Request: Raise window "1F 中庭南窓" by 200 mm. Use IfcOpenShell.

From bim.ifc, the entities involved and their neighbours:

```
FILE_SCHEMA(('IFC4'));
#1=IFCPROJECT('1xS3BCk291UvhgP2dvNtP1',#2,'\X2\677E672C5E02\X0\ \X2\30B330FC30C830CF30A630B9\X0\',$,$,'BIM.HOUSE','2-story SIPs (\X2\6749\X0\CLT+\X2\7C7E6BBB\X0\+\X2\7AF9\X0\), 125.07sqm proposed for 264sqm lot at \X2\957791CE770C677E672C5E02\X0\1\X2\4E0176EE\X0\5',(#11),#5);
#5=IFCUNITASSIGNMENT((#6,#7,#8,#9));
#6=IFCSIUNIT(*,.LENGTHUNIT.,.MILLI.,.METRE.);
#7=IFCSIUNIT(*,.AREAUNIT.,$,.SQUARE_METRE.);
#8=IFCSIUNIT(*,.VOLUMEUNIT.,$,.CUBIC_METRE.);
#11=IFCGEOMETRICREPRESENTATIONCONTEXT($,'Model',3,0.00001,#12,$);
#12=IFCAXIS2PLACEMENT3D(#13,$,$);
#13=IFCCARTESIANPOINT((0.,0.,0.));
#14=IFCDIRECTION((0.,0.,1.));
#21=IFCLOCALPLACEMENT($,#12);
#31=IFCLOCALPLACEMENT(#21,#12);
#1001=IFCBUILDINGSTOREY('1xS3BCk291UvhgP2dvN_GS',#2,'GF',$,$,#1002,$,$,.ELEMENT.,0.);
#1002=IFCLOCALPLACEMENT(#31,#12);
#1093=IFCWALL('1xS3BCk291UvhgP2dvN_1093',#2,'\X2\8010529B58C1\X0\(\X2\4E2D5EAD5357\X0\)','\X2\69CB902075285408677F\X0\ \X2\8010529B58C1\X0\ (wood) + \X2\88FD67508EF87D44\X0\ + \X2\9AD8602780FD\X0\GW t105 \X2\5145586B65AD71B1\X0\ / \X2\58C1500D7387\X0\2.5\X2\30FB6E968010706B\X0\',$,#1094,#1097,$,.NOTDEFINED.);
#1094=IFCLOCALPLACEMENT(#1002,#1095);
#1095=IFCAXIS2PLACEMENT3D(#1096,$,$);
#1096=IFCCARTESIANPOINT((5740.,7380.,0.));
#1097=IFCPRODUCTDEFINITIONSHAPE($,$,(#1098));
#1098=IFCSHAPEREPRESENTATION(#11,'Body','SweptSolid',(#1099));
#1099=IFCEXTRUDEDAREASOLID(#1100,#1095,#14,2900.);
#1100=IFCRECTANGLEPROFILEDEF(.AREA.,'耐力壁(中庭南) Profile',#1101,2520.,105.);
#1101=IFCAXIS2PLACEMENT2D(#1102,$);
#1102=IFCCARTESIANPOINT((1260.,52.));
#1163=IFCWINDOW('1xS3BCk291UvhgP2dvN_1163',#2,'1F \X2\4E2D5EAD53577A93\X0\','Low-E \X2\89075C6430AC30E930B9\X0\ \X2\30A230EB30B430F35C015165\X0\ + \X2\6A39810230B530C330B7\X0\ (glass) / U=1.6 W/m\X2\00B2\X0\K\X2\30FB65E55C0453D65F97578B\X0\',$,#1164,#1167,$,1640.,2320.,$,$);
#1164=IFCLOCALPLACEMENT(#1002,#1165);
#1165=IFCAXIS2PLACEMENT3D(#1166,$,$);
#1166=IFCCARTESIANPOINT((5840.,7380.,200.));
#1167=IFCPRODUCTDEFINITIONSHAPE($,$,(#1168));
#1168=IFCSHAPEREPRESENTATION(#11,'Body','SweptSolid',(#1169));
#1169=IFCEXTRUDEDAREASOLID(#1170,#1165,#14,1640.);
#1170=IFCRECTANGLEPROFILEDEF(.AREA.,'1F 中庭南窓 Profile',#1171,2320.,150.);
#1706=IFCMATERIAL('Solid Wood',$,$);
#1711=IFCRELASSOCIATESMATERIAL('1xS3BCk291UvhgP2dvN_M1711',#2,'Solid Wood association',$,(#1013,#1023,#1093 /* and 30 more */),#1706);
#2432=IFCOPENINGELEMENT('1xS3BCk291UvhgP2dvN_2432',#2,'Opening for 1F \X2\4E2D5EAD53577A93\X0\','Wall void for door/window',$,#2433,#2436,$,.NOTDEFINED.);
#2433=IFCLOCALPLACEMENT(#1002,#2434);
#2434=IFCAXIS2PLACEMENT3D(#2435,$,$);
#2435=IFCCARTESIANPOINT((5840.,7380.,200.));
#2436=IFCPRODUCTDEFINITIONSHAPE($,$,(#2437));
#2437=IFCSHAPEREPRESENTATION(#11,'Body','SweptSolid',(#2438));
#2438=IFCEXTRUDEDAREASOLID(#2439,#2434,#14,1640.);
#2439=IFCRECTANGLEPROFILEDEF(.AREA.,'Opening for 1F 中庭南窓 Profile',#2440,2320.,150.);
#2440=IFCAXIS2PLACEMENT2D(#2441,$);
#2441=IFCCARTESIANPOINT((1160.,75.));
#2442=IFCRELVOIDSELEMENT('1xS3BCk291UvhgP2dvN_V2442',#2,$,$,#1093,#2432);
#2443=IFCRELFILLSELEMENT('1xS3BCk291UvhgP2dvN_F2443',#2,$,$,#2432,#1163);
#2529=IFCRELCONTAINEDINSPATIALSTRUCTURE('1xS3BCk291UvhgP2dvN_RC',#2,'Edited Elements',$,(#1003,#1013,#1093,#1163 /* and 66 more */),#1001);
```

```python
import numpy as np
import ifcopenshell
import ifcopenshell.api.geometry
import ifcopenshell.util.placement
import ifcopenshell.util.unit

model = ifcopenshell.open("bim.ifc")
unit_scale = ifcopenshell.util.unit.calculate_unit_scale(model)

window = model.by_guid("1xS3BCk291UvhgP2dvN_1163")
opening = window.FillsVoids[0].RelatingOpeningElement
dz = 0.2 / unit_scale

shift = np.array([0.0, 0.0, dz])
# The window is not placed relative to its opening, so move both.
for product in (opening, window):
    matrix = ifcopenshell.util.placement.get_local_placement(product.ObjectPlacement)
    matrix[:3, 3] += shift
    ifcopenshell.api.geometry.edit_object_placement(model, product=product, matrix=matrix, is_si=False)

print(f"moved by {dz * unit_scale:+.3f} m")

model.write("bim_rev.ifc")
```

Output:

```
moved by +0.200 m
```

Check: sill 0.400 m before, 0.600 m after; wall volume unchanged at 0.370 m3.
